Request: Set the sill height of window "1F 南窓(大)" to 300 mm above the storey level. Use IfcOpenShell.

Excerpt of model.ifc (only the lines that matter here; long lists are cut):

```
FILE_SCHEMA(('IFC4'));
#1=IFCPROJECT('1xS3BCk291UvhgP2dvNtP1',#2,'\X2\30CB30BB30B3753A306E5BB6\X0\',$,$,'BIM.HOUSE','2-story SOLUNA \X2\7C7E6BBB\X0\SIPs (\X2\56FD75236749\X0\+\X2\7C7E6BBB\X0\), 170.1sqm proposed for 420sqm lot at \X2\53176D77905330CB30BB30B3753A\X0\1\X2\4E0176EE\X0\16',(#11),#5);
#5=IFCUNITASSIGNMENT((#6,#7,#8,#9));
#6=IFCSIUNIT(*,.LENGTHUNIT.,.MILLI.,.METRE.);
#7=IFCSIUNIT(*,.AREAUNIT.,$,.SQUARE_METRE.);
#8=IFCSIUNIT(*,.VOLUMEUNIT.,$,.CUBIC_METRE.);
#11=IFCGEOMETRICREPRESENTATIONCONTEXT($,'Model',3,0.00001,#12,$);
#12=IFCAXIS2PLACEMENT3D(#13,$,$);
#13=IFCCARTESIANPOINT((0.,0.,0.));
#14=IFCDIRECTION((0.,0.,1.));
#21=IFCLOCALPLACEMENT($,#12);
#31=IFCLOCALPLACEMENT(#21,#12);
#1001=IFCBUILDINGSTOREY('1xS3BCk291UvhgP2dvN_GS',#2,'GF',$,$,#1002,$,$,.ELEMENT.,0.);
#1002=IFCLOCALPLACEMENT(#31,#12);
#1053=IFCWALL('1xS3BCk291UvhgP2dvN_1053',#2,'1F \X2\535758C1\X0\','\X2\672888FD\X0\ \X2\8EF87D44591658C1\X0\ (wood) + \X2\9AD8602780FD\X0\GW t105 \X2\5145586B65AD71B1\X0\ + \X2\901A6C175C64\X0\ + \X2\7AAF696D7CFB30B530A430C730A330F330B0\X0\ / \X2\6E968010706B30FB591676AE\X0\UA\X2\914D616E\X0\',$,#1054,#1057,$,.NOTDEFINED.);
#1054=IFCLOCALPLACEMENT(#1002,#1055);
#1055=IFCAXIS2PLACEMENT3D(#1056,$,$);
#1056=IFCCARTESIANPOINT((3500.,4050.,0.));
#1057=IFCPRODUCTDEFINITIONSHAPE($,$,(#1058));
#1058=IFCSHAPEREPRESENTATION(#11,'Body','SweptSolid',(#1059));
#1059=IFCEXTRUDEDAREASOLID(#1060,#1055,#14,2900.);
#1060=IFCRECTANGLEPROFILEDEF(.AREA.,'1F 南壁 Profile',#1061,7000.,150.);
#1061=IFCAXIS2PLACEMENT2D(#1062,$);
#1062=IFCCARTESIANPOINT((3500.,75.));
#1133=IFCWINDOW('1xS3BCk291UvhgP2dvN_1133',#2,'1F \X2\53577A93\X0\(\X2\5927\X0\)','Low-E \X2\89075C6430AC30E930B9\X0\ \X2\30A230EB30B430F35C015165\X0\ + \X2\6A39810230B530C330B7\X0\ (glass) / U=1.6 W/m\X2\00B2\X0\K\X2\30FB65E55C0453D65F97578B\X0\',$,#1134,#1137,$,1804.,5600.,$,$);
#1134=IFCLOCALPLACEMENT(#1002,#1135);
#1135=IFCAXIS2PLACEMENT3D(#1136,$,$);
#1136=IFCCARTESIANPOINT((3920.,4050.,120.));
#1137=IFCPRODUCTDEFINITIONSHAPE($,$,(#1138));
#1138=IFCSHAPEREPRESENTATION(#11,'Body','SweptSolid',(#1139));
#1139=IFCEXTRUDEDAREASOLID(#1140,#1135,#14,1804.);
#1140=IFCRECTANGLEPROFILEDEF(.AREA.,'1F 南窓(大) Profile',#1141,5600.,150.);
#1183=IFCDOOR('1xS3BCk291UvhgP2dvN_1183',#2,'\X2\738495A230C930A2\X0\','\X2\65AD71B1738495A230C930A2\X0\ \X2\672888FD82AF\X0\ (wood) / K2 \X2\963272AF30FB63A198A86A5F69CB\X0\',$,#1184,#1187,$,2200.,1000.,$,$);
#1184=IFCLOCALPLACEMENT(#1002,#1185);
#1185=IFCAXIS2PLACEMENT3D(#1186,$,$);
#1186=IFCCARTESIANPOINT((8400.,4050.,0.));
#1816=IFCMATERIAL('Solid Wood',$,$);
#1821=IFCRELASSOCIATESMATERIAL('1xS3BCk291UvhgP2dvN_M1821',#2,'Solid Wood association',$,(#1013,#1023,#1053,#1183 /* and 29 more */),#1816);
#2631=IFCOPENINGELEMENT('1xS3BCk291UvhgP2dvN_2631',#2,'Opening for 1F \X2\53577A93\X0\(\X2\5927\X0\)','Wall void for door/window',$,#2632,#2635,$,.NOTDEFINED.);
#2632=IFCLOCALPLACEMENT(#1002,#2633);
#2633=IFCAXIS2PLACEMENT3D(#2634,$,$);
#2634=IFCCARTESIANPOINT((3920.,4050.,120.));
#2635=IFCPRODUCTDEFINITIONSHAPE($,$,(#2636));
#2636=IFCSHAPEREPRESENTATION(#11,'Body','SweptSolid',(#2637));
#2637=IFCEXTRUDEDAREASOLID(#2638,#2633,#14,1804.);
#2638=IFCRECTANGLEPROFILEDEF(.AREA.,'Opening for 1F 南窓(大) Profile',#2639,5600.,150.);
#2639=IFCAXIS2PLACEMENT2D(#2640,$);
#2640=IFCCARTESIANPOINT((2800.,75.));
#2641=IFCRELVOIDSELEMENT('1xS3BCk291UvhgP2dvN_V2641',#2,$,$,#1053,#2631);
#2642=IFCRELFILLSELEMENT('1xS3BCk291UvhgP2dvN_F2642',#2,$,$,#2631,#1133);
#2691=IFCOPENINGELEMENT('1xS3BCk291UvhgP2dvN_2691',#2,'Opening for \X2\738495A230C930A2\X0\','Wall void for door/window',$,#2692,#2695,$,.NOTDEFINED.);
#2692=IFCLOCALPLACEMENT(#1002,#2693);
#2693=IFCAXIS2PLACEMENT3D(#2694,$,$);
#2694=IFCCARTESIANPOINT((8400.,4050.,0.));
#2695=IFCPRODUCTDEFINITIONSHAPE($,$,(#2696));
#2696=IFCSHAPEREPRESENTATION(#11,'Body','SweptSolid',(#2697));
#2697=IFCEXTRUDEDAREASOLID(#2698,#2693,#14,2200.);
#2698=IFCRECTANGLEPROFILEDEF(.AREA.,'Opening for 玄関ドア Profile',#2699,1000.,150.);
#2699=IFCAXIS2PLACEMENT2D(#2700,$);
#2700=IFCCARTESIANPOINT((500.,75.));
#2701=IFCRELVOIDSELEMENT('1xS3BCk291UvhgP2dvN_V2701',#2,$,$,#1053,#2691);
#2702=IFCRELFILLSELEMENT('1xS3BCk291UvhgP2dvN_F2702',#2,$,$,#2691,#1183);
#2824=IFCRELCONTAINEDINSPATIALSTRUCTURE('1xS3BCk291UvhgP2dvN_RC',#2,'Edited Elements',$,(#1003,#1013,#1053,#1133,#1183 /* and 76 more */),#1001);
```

```python
import numpy as np
import ifcopenshell
import ifcopenshell.api.geometry
import ifcopenshell.geom
import ifcopenshell.util.element
import ifcopenshell.util.placement
import ifcopenshell.util.shape
import ifcopenshell.util.unit

model = ifcopenshell.open("model.ifc")
unit_scale = ifcopenshell.util.unit.calculate_unit_scale(model)

window = model.by_guid("1xS3BCk291UvhgP2dvN_1133")
opening = window.FillsVoids[0].RelatingOpeningElement
storey = ifcopenshell.util.element.get_container(window, ifc_class="IfcBuildingStorey")
level = ifcopenshell.util.placement.get_local_placement(storey.ObjectPlacement)[2, 3]

# The opening's origin need not be at the sill, so measure its lowest point.
shape = ifcopenshell.geom.create_shape(ifcopenshell.geom.settings(), opening)
bottom = ifcopenshell.util.shape.get_shape_bottom_elevation(shape, shape.geometry) / unit_scale
dz = level + 300.0 - bottom

shift = np.array([0.0, 0.0, dz])
# The window is not placed relative to its opening, so move both.
for product in (opening, window):
    matrix = ifcopenshell.util.placement.get_local_placement(product.ObjectPlacement)
    matrix[:3, 3] += shift
    ifcopenshell.api.geometry.edit_object_placement(model, product=product, matrix=matrix, is_si=False)

print(f"moved by {dz * unit_scale:+.3f} m")

model.write("model_updated.ifc")
```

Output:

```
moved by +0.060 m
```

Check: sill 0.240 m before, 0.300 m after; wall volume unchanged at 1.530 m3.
